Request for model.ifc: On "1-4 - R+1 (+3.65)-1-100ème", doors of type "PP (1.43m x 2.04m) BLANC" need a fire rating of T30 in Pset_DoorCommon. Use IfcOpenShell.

First a look at what the model holds.

```python
import ifcopenshell
import ifcopenshell.util.element

model = ifcopenshell.open("model.ifc")
print(model.schema)
storey = next(s for s in model.by_type("IfcBuildingStorey") if s.Name == "1-4 - R+1 (+3.65)-1-100ème")
doors = [e for e in ifcopenshell.util.element.get_decomposition(storey) if e.is_a("IfcDoor")]
seen = {}
for e in doors:
    element_type = ifcopenshell.util.element.get_type(e)
    key = (element_type.Name if element_type != e and element_type else None, ifcopenshell.util.element.get_pset(e, "Pset_DoorCommon", "FireRating"))
    seen[key] = seen.get(key, 0) + 1
for (name, value), count in sorted(seen.items(), key=str):
    print(count, "x", name, "|", value)
```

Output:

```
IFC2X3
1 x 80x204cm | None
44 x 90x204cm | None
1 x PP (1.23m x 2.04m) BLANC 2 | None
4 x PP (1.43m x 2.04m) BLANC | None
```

```python
import ifcopenshell
import ifcopenshell.api.pset
import ifcopenshell.util.element

model = ifcopenshell.open("model.ifc")

storey = next(s for s in model.by_type("IfcBuildingStorey") if s.Name == "1-4 - R+1 (+3.65)-1-100ème")
doors = [e for e in ifcopenshell.util.element.get_decomposition(storey) if e.is_a("IfcDoor")]

count = 0
for e in doors:
    element_type = ifcopenshell.util.element.get_type(e)
    if element_type in (None, e) or element_type.Name != "PP (1.43m x 2.04m) BLANC":
        continue
    # add_pset returns the element's existing set when there is one.
    pset = ifcopenshell.api.pset.add_pset(model, product=e, name="Pset_DoorCommon")
    ifcopenshell.api.pset.edit_pset(model, pset=pset, properties={"FireRating": "T30"})
    count += 1

print(count, "doors updated")

model.write("model_edited.ifc")
```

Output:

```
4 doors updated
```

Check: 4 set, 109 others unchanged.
